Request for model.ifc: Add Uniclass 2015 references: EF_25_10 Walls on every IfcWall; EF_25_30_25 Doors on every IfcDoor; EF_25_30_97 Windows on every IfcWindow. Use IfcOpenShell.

First a look at what the model holds.

```python
import ifcopenshell

model = ifcopenshell.open("model.ifc")
print(model.schema)
print("classifications:", [c.Name for c in model.by_type("IfcClassification")])
for ifc_class in ("IfcDoor", "IfcRoof", "IfcStair", "IfcWall", "IfcWindow"):
    print(ifc_class, len(model.by_type(ifc_class)))
```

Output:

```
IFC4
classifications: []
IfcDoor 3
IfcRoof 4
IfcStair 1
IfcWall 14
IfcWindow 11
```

```python
import ifcopenshell
import ifcopenshell.api.classification

model = ifcopenshell.open("model.ifc")

system = ifcopenshell.api.classification.add_classification(model, classification="Uniclass 2015")

codes = {
    "IfcWall": ("EF_25_10", "Walls"),
    "IfcDoor": ("EF_25_30_25", "Doors"),
    "IfcWindow": ("EF_25_30_97", "Windows"),
}
for ifc_class, (code, name) in codes.items():
    products = model.by_type(ifc_class)
    ifcopenshell.api.classification.add_reference(
        model, products=products, classification=system, identification=code, name=name
    )
    print(code, len(products))

model.write("model_v2.ifc")
```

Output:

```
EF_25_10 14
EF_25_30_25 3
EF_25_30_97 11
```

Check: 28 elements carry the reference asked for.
